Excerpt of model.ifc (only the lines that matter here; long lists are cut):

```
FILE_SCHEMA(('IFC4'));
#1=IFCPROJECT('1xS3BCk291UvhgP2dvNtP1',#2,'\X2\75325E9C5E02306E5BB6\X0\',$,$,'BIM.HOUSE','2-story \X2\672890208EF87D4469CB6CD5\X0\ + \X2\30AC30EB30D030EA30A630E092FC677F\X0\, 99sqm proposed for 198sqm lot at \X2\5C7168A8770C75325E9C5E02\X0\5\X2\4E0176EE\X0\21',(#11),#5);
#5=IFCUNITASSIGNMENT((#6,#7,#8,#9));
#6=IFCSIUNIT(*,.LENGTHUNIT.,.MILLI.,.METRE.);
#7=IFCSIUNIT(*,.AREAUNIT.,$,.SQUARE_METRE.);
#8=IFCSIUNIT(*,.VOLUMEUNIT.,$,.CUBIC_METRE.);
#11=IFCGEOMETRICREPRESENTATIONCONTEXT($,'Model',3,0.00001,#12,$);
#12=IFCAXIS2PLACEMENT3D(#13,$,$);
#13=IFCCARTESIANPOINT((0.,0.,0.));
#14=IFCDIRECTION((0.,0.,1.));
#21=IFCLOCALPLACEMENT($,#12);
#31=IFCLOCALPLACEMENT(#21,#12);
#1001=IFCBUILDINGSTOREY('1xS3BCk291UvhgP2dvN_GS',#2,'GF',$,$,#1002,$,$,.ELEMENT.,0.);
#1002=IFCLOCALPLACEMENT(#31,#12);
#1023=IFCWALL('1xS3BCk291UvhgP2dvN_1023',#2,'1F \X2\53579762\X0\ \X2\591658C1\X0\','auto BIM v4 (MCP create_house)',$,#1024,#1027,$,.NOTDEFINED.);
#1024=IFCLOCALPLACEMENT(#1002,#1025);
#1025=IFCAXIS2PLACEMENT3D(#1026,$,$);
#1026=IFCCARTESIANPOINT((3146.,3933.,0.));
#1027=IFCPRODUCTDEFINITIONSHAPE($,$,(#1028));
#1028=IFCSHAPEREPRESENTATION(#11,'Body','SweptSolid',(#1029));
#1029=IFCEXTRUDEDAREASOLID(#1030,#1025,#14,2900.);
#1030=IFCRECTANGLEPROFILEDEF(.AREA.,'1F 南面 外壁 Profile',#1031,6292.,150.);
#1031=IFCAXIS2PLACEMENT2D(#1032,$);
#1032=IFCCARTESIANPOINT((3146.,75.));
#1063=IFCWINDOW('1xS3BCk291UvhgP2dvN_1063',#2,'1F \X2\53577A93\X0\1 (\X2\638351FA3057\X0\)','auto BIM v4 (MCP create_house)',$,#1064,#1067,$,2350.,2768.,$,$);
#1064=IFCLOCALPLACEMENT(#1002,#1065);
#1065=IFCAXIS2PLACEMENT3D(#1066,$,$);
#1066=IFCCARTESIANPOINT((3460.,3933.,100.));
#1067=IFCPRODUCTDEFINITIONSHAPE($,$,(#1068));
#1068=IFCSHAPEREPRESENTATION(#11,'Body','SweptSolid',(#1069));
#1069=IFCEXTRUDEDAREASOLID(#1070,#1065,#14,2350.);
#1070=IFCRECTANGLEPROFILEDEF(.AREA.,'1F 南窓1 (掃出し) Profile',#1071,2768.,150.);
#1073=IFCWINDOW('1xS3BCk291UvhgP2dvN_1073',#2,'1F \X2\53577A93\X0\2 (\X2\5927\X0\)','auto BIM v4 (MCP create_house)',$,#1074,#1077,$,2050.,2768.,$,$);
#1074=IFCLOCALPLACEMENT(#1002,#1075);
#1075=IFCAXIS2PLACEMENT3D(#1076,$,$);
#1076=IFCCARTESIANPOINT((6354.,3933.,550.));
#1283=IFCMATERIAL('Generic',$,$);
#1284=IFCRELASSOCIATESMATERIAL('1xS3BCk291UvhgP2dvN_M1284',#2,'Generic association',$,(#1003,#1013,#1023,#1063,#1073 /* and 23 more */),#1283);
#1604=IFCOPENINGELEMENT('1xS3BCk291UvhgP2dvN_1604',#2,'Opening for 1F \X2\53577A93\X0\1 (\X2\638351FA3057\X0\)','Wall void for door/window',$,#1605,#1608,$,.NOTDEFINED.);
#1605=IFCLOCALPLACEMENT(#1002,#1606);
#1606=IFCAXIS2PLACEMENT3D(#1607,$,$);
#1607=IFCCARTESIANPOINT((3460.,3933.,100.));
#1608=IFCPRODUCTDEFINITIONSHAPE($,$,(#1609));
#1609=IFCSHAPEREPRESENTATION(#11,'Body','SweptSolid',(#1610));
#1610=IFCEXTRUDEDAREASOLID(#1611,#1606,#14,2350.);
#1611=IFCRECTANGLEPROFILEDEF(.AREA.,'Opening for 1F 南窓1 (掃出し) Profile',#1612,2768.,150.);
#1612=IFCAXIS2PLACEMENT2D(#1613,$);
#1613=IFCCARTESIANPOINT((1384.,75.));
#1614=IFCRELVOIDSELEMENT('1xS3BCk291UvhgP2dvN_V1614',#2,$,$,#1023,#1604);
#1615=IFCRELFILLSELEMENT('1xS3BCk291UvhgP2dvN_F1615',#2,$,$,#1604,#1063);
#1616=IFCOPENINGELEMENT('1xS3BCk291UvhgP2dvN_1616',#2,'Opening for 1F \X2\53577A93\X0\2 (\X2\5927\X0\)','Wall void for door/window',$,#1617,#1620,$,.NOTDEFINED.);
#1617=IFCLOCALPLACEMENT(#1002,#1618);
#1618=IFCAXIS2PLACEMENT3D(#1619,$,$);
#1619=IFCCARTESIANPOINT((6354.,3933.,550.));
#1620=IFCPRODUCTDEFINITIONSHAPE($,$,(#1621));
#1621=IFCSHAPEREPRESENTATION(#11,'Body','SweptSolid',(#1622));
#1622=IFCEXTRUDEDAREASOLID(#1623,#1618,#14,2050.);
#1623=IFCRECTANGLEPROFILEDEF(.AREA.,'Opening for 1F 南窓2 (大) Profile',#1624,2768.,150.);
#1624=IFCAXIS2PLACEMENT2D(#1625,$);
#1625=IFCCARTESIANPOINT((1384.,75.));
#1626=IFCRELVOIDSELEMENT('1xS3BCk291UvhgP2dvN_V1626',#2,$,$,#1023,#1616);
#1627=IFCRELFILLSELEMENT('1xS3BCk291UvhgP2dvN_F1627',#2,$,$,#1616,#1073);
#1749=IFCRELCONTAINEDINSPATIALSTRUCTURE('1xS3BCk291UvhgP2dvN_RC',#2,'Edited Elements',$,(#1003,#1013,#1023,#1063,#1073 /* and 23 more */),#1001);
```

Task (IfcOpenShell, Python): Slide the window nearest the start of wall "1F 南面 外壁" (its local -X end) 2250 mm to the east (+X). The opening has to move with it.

```python
import ifcopenshell
import ifcopenshell.api.geometry
import ifcopenshell.util.placement
import ifcopenshell.util.unit

model = ifcopenshell.open("model.ifc")
unit_scale = ifcopenshell.util.unit.calculate_unit_scale(model)

window = model.by_id(1063)
opening = window.FillsVoids[0].RelatingOpeningElement
wall = opening.VoidsElements[0].RelatingBuildingElement

wall_matrix = ifcopenshell.util.placement.get_local_placement(wall.ObjectPlacement)
shift = wall_matrix[:3, 0] * 2.25 / unit_scale
before = ifcopenshell.util.placement.get_local_placement(window.ObjectPlacement)[:3, 3].copy()

# The window is not placed relative to its opening, so move both.
for product in (opening, window):
    matrix = ifcopenshell.util.placement.get_local_placement(product.ObjectPlacement)
    matrix[:3, 3] += shift
    ifcopenshell.api.geometry.edit_object_placement(model, product=product, matrix=matrix, is_si=False)

after = ifcopenshell.util.placement.get_local_placement(window.ObjectPlacement)[:3, 3]
print("window moved by", (after - before).round(3) + 0.0)

model.write("model_edited.ifc")
```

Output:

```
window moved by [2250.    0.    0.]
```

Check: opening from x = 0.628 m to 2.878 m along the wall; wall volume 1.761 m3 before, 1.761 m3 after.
